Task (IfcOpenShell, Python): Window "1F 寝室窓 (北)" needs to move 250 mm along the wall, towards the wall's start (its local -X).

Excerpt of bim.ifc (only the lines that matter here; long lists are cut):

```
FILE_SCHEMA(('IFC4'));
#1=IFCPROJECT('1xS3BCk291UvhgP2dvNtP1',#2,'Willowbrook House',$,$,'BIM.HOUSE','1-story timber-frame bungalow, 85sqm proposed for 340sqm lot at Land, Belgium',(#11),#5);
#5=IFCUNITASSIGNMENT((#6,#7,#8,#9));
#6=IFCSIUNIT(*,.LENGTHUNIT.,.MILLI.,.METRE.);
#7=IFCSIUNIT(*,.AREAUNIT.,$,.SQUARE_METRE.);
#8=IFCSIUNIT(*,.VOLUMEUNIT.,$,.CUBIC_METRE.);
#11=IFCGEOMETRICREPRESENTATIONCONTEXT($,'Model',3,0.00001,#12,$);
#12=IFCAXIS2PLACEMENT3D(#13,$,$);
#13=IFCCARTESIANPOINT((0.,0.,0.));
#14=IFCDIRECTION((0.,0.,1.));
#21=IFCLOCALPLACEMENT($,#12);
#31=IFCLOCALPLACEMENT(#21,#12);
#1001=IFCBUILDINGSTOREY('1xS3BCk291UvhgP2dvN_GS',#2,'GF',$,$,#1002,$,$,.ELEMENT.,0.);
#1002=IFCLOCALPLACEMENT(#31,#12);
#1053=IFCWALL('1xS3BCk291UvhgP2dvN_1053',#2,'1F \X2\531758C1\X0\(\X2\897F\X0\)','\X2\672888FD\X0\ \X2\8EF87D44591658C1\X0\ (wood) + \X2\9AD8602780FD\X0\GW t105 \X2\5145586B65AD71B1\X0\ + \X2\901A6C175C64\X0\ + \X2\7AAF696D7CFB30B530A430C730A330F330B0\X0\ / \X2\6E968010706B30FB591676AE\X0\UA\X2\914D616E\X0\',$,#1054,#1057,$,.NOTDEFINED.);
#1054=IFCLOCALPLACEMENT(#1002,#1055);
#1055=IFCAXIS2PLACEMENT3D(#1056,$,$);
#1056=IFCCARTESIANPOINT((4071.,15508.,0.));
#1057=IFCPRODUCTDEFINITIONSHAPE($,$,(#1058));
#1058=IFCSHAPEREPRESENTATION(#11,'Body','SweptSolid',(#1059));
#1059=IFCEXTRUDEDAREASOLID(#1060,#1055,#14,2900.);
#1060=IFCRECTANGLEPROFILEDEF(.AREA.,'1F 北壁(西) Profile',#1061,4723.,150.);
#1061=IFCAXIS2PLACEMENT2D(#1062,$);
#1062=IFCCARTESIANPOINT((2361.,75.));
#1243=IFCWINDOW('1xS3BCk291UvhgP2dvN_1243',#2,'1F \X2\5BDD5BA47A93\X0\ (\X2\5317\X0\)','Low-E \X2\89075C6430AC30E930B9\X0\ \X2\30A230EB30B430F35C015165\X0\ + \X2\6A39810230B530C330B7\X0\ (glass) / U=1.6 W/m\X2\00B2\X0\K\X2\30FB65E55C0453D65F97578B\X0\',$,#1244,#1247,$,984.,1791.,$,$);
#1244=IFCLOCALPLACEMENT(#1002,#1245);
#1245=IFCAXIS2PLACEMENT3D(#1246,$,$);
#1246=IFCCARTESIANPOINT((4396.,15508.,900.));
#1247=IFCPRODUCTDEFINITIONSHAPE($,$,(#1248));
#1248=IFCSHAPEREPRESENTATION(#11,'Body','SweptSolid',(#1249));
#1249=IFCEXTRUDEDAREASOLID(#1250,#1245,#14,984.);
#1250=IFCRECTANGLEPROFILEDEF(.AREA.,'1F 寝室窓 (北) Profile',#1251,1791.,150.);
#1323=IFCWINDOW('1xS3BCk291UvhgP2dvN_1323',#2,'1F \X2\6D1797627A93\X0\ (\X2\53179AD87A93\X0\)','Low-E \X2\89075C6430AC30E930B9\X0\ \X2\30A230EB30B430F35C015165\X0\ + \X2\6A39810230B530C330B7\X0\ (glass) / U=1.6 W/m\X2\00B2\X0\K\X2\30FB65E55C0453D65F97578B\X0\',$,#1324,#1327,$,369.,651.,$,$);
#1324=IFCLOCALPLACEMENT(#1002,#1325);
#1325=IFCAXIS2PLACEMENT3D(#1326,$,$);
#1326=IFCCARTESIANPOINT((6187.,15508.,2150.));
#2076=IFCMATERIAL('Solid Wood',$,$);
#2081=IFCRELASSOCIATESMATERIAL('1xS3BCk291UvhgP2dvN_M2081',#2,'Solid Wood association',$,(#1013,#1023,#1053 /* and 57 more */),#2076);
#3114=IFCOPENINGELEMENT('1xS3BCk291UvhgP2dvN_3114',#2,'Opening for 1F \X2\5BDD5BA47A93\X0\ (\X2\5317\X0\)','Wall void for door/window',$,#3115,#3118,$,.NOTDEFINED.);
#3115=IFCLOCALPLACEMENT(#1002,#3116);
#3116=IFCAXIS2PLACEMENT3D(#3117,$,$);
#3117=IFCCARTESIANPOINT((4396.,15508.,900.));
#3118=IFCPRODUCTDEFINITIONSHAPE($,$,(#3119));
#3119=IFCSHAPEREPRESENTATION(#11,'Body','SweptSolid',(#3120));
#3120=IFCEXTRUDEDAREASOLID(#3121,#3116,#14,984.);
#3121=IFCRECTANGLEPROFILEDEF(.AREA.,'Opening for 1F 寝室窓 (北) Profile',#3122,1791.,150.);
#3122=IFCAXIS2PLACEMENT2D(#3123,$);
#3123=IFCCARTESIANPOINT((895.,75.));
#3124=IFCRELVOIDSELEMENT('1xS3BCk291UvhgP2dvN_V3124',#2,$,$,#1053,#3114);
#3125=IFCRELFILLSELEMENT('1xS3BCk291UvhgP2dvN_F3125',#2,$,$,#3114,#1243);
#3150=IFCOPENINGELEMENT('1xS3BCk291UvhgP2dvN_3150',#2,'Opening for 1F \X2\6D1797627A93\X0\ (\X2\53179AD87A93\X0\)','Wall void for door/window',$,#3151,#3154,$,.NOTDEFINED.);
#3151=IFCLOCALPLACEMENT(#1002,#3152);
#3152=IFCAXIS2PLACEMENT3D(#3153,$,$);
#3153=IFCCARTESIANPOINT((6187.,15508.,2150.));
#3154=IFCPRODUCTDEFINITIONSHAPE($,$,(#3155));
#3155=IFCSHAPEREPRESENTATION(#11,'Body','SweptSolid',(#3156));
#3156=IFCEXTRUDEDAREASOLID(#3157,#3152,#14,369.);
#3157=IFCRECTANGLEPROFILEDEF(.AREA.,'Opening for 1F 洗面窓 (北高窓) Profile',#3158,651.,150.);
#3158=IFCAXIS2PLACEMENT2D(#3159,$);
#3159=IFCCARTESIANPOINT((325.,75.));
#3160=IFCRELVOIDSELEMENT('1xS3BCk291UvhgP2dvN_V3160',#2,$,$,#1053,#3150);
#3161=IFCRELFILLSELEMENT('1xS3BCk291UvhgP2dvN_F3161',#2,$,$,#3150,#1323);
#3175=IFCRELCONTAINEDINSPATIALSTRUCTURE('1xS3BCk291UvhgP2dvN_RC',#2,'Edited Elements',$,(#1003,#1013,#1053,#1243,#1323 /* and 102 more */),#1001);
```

```python
import ifcopenshell
import ifcopenshell.api.geometry
import ifcopenshell.util.placement
import ifcopenshell.util.unit

model = ifcopenshell.open("bim.ifc")
unit_scale = ifcopenshell.util.unit.calculate_unit_scale(model)

window = model.by_guid("1xS3BCk291UvhgP2dvN_1243")
opening = window.FillsVoids[0].RelatingOpeningElement
wall = opening.VoidsElements[0].RelatingBuildingElement

wall_matrix = ifcopenshell.util.placement.get_local_placement(wall.ObjectPlacement)
shift = wall_matrix[:3, 0] * -0.25 / unit_scale
before = ifcopenshell.util.placement.get_local_placement(window.ObjectPlacement)[:3, 3].copy()

# The window is not placed relative to its opening, so move both.
for product in (opening, window):
    matrix = ifcopenshell.util.placement.get_local_placement(product.ObjectPlacement)
    matrix[:3, 3] += shift
    ifcopenshell.api.geometry.edit_object_placement(model, product=product, matrix=matrix, is_si=False)

after = ifcopenshell.util.placement.get_local_placement(window.ObjectPlacement)[:3, 3]
print("window moved by", (after - before).round(3) + 0.0)

model.write("bim_rev.ifc")
```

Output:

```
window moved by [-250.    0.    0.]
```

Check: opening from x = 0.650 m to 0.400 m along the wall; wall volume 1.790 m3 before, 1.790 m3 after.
